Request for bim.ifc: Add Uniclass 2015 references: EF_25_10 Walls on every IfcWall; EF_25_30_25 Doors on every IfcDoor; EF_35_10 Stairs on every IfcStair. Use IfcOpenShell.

First a look at what the model holds.

```python
import ifcopenshell

model = ifcopenshell.open("bim.ifc")
print(model.schema)
print("classifications:", [c.Name for c in model.by_type("IfcClassification")])
for ifc_class in ("IfcDoor", "IfcRoof", "IfcStair", "IfcWall", "IfcWindow"):
    print(ifc_class, len(model.by_type(ifc_class)))
```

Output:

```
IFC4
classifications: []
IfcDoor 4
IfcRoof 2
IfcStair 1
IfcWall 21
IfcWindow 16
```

```python
import ifcopenshell
import ifcopenshell.api.classification

model = ifcopenshell.open("bim.ifc")

system = ifcopenshell.api.classification.add_classification(model, classification="Uniclass 2015")

codes = {
    "IfcWall": ("EF_25_10", "Walls"),
    "IfcDoor": ("EF_25_30_25", "Doors"),
    "IfcStair": ("EF_35_10", "Stairs"),
}
for ifc_class, (code, name) in codes.items():
    products = model.by_type(ifc_class)
    ifcopenshell.api.classification.add_reference(
        model, products=products, classification=system, identification=code, name=name
    )
    print(code, len(products))

model.write("bim_updated.ifc")
```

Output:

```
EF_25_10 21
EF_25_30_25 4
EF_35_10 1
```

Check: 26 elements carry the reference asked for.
